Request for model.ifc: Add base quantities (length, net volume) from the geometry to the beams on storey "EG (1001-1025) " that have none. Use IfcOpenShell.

First a look at what the model holds.

```python
import ifcopenshell
import ifcopenshell.util.element
import ifcopenshell.util.unit

model = ifcopenshell.open("model.ifc")
print(model.schema)
for unit_type in ("LENGTHUNIT", "AREAUNIT", "VOLUMEUNIT"):
    print(unit_type, ifcopenshell.util.unit.calculate_unit_scale(model, unit_type))
storey = next(s for s in model.by_type("IfcBuildingStorey") if s.Name == "EG (1001-1025) ")
beams = [e for e in ifcopenshell.util.element.get_decomposition(storey) if e.is_a("IfcBeam")]
for e in sorted(beams, key=lambda e: e.id()):
    print(e.id(), e.is_a(), e.Name, list(ifcopenshell.util.element.get_psets(e, qtos_only=True)), sep=" | ")
```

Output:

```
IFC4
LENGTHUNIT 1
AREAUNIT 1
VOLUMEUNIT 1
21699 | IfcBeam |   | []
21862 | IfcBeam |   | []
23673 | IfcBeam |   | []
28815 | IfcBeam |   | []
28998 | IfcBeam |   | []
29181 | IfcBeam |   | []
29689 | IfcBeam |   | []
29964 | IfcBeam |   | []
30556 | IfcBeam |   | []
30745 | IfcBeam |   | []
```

```python
import ifcopenshell
import ifcopenshell.api.pset
import ifcopenshell.geom
import ifcopenshell.util.element
import ifcopenshell.util.shape
import ifcopenshell.util.unit

model = ifcopenshell.open("model.ifc")
unit_scale = ifcopenshell.util.unit.calculate_unit_scale(model)
volume_scale = ifcopenshell.util.unit.calculate_unit_scale(model, "VOLUMEUNIT")
settings = ifcopenshell.geom.settings()

storey = next(s for s in model.by_type("IfcBuildingStorey") if s.Name == "EG (1001-1025) ")
beams = [e for e in ifcopenshell.util.element.get_decomposition(storey) if e.is_a("IfcBeam")]

for e in sorted(beams, key=lambda e: e.id()):
    if ifcopenshell.util.element.get_psets(e, qtos_only=True, should_inherit=False):
        continue
    # Geometry comes back in metres, in the element's own axes.
    shape = ifcopenshell.geom.create_shape(settings, e)
    values = {
        "Length": ifcopenshell.util.shape.get_max_xyz(shape.geometry) / unit_scale,
        "NetVolume": ifcopenshell.util.shape.get_volume(shape.geometry) / volume_scale,
    }
    qto = ifcopenshell.api.pset.add_qto(model, product=e, name="Qto_BeamBaseQuantities")
    ifcopenshell.api.pset.edit_qto(model, qto=qto, properties=values)
    print(e.id(), {k: round(v, 3) for k, v in values.items()})

model.write("model_v2.ifc")
```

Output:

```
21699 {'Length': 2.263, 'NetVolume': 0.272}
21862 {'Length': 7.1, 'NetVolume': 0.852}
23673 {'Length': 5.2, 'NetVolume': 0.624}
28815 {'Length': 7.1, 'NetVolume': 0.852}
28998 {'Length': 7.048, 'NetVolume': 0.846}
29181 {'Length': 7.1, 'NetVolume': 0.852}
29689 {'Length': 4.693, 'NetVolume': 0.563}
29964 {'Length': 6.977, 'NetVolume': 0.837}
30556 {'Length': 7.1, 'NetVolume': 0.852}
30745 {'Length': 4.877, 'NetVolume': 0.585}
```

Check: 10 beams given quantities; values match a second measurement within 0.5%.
